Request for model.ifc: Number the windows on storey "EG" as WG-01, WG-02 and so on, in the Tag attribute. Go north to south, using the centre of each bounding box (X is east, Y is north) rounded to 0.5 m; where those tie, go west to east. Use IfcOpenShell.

First a look at what the model holds.

```python
import ifcopenshell
import ifcopenshell.util.element
import ifcopenshell.util.placement

model = ifcopenshell.open("model.ifc")
print(model.schema)
storey = next(s for s in model.by_type("IfcBuildingStorey") if s.Name == "EG")
windows = [e for e in ifcopenshell.util.element.get_decomposition(storey) if e.is_a("IfcWindow")]
for e in sorted(windows, key=lambda e: e.id()):
    origin = ifcopenshell.util.placement.get_local_placement(e.ObjectPlacement)[:3, 3]
    print(e.id(), e.Tag, e.Name, origin.round(2) + 0.0, sep=" | ")
```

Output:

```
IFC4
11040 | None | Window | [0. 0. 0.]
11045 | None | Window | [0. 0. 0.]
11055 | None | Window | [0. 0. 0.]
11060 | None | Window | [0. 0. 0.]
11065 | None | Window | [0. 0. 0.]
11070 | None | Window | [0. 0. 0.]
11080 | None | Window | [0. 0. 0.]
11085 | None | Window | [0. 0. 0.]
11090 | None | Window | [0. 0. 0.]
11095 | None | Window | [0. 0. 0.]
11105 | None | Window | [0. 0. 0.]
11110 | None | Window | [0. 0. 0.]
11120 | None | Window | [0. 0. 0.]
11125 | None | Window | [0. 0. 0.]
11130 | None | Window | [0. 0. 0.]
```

```python
import ifcopenshell
import ifcopenshell.geom
import ifcopenshell.util.element
import ifcopenshell.util.shape

model = ifcopenshell.open("model.ifc")
settings = ifcopenshell.geom.settings()
settings.set("use-world-coords", True)


def centre(element):
    shape = ifcopenshell.geom.create_shape(settings, element)
    return ifcopenshell.util.shape.get_bbox_centroid(shape.geometry)


storey = next(s for s in model.by_type("IfcBuildingStorey") if s.Name == "EG")
windows = [e for e in ifcopenshell.util.element.get_decomposition(storey) if e.is_a("IfcWindow")]

# Insertion points can sit at a corner or the storey origin, so sort by the geometry (in metres).
centres = {e: centre(e) for e in windows}
windows.sort(key=lambda e: (-round(centres[e][1] / 0.5), centres[e][0]))

for i, e in enumerate(windows, start=1):
    number = f"WG-{i:02d}"
    e.Tag = number
    print(e.id(), number)

model.write("model_v2.ifc")
```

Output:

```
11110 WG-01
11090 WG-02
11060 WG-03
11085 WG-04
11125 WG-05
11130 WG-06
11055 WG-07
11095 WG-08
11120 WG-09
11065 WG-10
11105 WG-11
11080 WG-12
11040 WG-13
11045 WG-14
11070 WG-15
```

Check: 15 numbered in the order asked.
